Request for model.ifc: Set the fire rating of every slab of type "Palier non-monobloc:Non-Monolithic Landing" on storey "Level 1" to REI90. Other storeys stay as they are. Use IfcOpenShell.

First a look at what the model holds.

```python
import ifcopenshell
import ifcopenshell.util.element

model = ifcopenshell.open("model.ifc")
print(model.schema)
storey = next(s for s in model.by_type("IfcBuildingStorey") if s.Name == "Level 1")
slabs = [e for e in ifcopenshell.util.element.get_decomposition(storey) if e.is_a("IfcSlab")]
seen = {}
for e in slabs:
    element_type = ifcopenshell.util.element.get_type(e)
    key = (element_type.Name if element_type != e and element_type else None, ifcopenshell.util.element.get_pset(e, "Pset_SlabCommon", "FireRating"))
    seen[key] = seen.get(key, 0) + 1
for (name, value), count in sorted(seen.items(), key=str):
    print(count, "x", name, "|", value)
```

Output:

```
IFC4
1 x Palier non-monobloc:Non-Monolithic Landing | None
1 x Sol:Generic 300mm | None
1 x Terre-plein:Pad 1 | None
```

```python
import ifcopenshell
import ifcopenshell.api.pset
import ifcopenshell.util.element

model = ifcopenshell.open("model.ifc")

storey = next(s for s in model.by_type("IfcBuildingStorey") if s.Name == "Level 1")
slabs = [e for e in ifcopenshell.util.element.get_decomposition(storey) if e.is_a("IfcSlab")]

count = 0
for e in slabs:
    element_type = ifcopenshell.util.element.get_type(e)
    if element_type in (None, e) or element_type.Name != "Palier non-monobloc:Non-Monolithic Landing":
        continue
    # add_pset returns the element's existing set when there is one.
    pset = ifcopenshell.api.pset.add_pset(model, product=e, name="Pset_SlabCommon")
    ifcopenshell.api.pset.edit_pset(model, pset=pset, properties={"FireRating": "REI90"})
    count += 1

print(count, "slabs updated")

model.write("model_updated.ifc")
```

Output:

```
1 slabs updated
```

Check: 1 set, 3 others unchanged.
